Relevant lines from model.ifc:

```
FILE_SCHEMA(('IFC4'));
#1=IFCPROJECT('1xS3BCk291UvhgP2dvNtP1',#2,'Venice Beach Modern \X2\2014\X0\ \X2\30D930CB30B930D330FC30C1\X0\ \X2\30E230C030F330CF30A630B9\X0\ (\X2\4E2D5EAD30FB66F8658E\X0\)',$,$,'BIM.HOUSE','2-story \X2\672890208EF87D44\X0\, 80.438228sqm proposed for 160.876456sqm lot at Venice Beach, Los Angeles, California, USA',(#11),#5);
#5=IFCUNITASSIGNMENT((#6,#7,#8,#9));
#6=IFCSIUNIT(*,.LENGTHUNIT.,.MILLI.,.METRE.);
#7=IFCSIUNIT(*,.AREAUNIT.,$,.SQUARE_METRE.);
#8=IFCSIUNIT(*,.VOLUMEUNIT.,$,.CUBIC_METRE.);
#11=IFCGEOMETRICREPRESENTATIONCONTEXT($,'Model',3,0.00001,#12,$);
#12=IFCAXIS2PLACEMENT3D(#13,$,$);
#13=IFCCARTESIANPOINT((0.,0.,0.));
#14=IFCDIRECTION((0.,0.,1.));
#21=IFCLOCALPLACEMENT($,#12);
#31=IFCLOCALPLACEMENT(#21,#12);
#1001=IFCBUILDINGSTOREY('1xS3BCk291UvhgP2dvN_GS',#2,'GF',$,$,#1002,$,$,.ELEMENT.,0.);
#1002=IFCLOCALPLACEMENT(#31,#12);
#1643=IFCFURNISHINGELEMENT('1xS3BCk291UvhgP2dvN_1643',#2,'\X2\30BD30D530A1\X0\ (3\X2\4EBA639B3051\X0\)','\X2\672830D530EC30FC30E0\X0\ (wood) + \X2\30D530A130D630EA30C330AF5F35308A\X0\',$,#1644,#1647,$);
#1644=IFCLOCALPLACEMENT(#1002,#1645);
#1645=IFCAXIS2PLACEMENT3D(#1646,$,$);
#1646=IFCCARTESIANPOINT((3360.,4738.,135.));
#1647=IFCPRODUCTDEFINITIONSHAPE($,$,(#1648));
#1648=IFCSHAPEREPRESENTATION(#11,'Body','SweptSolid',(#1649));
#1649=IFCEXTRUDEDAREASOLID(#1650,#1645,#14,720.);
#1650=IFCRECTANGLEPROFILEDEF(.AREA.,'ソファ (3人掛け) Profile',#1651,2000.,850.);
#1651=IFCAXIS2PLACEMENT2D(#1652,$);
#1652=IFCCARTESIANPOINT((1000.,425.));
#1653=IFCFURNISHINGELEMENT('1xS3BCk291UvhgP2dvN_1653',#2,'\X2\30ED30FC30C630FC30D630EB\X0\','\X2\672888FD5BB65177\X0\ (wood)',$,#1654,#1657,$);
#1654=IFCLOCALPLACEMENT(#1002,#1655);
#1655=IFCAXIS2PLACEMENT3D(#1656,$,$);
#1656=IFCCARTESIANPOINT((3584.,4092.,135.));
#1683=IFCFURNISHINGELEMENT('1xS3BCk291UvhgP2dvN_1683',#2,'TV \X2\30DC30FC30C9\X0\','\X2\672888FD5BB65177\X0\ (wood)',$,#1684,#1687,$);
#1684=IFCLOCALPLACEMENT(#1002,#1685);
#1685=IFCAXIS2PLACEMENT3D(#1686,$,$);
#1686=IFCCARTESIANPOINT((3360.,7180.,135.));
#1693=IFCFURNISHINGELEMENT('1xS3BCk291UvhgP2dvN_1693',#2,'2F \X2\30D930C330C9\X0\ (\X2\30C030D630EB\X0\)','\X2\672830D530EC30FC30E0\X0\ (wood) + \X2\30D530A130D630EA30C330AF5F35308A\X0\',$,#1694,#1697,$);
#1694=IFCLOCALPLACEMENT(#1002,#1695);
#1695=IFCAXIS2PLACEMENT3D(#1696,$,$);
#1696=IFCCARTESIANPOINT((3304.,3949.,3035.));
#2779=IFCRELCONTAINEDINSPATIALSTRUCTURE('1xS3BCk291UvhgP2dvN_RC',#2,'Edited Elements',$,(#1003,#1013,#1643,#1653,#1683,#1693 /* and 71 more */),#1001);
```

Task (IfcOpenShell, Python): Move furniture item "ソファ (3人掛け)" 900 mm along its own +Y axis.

```python
import ifcopenshell
import ifcopenshell.api.geometry
import ifcopenshell.util.placement

model = ifcopenshell.open("model.ifc")

item = model.by_guid("1xS3BCk291UvhgP2dvN_1643")
matrix = ifcopenshell.util.placement.get_local_placement(item.ObjectPlacement)
matrix[:3, 3] += matrix[:3, 1] * 900.0
ifcopenshell.api.geometry.edit_object_placement(model, product=item, matrix=matrix, is_si=False)

print(ifcopenshell.util.placement.get_local_placement(item.ObjectPlacement).round(3) + 0.0)

model.write("model_edited.ifc")
```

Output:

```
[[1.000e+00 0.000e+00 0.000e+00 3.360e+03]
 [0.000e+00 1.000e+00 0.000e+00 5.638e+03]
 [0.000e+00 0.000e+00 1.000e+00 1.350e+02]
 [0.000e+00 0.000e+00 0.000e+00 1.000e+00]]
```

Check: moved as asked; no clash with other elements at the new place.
